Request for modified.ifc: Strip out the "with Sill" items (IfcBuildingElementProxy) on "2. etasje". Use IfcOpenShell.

First a look at what the model holds.

```python
import ifcopenshell
import ifcopenshell.util.element

model = ifcopenshell.open("modified.ifc")
print(model.schema)
storey = next(s for s in model.by_type("IfcBuildingStorey") if s.Name == "2. etasje")
proxies = [e for e in ifcopenshell.util.element.get_decomposition(storey) if e.is_a("IfcBuildingElementProxy")]
seen = {}
for e in proxies:
    element_type = ifcopenshell.util.element.get_type(e)
    name = element_type.Name if element_type not in (None, e) else None
    seen[name] = seen.get(name, 0) + 1
for name, count in sorted(seen.items(), key=str):
    print(count, "x", name)
```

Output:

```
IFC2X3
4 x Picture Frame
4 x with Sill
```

```python
import ifcopenshell
import ifcopenshell.api.root
import ifcopenshell.util.element

model = ifcopenshell.open("modified.ifc")

storey = next(s for s in model.by_type("IfcBuildingStorey") if s.Name == "2. etasje")
proxies = [e for e in ifcopenshell.util.element.get_decomposition(storey) if e.is_a("IfcBuildingElementProxy")]
targets = [e for e in proxies if (t := ifcopenshell.util.element.get_type(e)) not in (None, e) and t.Name == "with Sill"]

for e in targets:
    ifcopenshell.api.root.remove_product(model, product=e)
print(len(targets), "removed")

model.write("modified_v2.ifc")
```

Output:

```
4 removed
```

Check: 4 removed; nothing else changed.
